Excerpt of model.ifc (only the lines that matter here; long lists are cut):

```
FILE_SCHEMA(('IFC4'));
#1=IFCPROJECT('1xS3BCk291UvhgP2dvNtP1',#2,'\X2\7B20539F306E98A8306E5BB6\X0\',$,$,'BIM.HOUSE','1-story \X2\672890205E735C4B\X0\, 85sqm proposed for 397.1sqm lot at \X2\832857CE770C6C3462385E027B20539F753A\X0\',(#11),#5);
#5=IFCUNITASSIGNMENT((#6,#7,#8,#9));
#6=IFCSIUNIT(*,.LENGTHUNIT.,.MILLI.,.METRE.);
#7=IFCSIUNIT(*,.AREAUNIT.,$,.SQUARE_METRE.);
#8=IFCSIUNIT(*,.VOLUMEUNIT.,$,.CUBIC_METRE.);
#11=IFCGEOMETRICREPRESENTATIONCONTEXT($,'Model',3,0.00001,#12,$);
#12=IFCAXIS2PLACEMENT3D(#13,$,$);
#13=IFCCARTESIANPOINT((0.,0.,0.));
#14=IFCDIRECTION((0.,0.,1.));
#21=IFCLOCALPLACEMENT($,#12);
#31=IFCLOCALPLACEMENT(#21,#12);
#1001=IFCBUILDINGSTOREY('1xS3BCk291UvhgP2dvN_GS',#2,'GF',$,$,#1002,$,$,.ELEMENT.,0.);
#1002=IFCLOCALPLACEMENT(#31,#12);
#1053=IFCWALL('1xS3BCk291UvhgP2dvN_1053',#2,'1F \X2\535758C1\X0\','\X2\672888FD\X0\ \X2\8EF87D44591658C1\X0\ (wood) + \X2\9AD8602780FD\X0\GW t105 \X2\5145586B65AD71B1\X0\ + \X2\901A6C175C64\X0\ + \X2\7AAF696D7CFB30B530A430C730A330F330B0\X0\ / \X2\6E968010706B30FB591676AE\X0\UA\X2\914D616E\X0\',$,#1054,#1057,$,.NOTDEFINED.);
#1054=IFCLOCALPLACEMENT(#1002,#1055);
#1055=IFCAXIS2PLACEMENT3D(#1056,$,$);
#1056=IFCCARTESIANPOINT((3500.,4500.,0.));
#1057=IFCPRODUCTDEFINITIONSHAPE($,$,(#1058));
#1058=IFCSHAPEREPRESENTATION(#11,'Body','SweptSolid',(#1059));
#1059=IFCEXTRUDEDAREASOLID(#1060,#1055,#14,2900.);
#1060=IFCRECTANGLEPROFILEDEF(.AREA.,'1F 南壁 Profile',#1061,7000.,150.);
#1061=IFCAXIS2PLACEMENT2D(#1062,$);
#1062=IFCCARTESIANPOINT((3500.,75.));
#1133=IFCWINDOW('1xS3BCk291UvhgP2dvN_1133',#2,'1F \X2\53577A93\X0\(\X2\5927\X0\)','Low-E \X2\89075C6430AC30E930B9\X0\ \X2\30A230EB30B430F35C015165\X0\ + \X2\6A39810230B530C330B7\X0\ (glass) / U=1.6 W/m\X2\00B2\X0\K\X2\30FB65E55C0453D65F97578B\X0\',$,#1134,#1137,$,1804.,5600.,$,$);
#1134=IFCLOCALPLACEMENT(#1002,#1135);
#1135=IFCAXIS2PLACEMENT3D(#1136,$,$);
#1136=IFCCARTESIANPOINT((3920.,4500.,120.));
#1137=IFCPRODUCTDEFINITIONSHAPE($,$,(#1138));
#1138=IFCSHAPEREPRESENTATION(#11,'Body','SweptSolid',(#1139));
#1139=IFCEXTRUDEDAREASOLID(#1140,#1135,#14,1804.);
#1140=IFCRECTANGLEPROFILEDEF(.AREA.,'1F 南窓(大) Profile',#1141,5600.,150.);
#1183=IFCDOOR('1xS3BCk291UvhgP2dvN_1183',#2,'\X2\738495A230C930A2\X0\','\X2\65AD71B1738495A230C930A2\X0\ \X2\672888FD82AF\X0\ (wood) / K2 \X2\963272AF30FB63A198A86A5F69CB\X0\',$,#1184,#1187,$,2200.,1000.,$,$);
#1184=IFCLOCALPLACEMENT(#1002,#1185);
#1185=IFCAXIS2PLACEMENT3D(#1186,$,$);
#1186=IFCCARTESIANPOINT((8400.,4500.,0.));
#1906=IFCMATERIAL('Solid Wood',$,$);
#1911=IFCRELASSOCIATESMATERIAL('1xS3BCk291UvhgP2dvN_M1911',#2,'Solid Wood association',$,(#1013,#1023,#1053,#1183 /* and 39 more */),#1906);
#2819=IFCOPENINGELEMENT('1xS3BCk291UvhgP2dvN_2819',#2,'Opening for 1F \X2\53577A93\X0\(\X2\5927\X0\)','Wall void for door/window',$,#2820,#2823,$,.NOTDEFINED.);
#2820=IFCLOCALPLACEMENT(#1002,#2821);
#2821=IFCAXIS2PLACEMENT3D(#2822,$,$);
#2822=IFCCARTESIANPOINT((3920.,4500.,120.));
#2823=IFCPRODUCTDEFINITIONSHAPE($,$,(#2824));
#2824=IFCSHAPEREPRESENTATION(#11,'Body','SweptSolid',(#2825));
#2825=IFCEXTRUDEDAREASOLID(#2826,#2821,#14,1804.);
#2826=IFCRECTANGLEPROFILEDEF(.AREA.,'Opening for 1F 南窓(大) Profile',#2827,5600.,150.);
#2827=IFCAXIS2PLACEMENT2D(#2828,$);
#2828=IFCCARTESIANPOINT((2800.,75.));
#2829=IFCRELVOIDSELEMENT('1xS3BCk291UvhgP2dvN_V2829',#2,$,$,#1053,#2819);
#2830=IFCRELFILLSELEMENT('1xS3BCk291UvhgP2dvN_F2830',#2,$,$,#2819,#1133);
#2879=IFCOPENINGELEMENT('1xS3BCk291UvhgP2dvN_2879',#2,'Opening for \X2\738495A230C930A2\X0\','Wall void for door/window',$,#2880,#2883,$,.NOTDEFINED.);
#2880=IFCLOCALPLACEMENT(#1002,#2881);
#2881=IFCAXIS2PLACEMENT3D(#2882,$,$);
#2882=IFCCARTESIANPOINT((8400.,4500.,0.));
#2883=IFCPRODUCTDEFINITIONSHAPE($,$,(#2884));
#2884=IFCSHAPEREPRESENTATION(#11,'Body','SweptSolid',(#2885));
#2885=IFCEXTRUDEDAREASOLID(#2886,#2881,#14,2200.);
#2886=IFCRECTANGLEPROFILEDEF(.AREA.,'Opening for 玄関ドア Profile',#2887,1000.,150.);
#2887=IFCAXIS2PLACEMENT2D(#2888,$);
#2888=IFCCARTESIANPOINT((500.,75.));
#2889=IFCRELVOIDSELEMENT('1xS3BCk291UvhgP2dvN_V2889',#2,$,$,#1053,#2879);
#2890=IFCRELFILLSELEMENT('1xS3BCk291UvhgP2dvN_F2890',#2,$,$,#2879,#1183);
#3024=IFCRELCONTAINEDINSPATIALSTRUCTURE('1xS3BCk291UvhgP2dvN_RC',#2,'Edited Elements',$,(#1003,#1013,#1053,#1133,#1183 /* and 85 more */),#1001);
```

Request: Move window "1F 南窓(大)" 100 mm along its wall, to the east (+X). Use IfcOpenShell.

```python
import ifcopenshell
import ifcopenshell.api.geometry
import ifcopenshell.util.placement
import ifcopenshell.util.unit

model = ifcopenshell.open("model.ifc")
unit_scale = ifcopenshell.util.unit.calculate_unit_scale(model)

window = model.by_guid("1xS3BCk291UvhgP2dvN_1133")
opening = window.FillsVoids[0].RelatingOpeningElement
wall = opening.VoidsElements[0].RelatingBuildingElement

wall_matrix = ifcopenshell.util.placement.get_local_placement(wall.ObjectPlacement)
shift = wall_matrix[:3, 0] * 0.1 / unit_scale
before = ifcopenshell.util.placement.get_local_placement(window.ObjectPlacement)[:3, 3].copy()

# The window is not placed relative to its opening, so move both.
for product in (opening, window):
    matrix = ifcopenshell.util.placement.get_local_placement(product.ObjectPlacement)
    matrix[:3, 3] += shift
    ifcopenshell.api.geometry.edit_object_placement(model, product=product, matrix=matrix, is_si=False)

after = ifcopenshell.util.placement.get_local_placement(window.ObjectPlacement)[:3, 3]
print("window moved by", (after - before).round(3) + 0.0)

model.write("model-out.ifc")
```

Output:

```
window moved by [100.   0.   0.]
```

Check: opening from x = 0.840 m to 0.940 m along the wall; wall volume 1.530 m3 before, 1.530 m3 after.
